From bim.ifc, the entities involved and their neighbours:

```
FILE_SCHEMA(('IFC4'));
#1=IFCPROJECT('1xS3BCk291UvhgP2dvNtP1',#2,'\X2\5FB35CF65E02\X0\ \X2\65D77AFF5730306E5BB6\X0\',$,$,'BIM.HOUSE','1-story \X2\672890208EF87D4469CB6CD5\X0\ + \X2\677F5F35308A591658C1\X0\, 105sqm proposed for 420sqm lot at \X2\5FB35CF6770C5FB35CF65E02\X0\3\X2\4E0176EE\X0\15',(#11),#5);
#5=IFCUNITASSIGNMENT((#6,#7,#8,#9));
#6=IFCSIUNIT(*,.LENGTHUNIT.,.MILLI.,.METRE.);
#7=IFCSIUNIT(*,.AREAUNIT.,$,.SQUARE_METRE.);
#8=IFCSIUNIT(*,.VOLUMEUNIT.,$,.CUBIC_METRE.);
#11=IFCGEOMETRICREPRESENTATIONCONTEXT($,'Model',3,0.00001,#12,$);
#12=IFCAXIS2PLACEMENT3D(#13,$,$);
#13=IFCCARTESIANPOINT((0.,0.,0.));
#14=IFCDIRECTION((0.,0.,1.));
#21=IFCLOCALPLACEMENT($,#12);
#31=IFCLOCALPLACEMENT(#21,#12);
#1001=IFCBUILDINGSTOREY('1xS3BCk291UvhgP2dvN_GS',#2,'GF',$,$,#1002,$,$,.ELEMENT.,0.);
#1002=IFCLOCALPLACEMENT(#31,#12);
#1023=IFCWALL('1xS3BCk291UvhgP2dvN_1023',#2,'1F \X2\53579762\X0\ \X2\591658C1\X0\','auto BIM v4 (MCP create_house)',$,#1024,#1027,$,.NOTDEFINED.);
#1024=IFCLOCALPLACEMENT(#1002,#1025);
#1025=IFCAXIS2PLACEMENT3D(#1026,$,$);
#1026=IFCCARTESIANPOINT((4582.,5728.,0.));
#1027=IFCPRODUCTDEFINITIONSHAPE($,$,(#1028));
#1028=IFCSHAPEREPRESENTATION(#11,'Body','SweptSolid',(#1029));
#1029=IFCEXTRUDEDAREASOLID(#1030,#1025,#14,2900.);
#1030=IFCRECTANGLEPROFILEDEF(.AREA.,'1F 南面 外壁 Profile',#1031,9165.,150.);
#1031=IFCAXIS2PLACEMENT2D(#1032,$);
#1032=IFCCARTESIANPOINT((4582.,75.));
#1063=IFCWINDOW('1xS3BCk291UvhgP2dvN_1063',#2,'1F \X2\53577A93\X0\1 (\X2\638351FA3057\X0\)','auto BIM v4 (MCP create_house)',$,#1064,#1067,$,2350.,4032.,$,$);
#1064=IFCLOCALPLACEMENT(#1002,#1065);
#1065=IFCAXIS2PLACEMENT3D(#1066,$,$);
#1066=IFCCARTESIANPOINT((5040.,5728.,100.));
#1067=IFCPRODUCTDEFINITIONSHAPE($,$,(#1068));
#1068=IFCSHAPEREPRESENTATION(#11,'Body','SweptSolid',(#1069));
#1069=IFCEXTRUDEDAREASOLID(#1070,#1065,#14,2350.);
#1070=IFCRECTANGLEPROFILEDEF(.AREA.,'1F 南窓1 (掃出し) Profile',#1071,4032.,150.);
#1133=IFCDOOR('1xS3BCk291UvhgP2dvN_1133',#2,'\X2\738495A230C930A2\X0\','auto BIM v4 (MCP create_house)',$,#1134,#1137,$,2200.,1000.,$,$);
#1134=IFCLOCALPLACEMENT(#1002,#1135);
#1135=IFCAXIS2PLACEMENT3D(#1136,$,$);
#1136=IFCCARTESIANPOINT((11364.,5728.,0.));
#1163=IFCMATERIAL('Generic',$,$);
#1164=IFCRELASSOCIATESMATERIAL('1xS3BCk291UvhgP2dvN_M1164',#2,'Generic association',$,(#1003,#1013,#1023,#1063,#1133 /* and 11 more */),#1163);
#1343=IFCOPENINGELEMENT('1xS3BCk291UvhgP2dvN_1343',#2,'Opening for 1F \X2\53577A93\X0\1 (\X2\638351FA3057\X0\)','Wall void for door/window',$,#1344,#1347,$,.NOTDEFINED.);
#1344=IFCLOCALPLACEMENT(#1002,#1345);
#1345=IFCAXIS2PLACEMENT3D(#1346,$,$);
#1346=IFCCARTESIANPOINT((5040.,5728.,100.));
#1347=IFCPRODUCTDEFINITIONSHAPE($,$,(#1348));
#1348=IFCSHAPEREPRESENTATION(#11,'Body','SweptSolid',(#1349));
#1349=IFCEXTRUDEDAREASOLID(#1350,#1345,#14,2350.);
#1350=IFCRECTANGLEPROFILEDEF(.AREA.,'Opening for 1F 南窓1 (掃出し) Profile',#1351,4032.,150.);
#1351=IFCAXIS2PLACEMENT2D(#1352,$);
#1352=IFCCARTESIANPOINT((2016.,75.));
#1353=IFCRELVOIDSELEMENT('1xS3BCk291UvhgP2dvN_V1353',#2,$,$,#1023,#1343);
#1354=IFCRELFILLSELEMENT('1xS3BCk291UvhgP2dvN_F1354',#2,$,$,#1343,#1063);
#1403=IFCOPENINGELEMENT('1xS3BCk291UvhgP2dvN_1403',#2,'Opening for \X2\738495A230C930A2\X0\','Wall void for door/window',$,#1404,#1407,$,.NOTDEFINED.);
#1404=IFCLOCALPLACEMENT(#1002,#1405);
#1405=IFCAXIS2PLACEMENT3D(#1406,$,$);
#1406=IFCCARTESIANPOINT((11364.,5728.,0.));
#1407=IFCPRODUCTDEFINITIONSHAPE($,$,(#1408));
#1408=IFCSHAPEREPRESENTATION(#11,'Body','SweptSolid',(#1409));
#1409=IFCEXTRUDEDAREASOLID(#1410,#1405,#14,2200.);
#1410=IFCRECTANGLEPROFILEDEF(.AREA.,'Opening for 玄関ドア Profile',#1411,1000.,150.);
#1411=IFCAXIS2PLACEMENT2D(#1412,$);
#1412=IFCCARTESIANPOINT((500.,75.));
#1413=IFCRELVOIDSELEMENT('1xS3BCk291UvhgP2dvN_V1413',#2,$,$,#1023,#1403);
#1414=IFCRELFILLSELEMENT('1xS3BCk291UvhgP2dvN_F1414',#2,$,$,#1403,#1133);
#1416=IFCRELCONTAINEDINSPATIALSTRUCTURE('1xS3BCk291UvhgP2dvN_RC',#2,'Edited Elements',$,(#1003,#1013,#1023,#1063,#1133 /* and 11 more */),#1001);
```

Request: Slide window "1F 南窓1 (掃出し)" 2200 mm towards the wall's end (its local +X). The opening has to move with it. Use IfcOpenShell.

```python
import ifcopenshell
import ifcopenshell.api.geometry
import ifcopenshell.util.placement
import ifcopenshell.util.unit

model = ifcopenshell.open("bim.ifc")
unit_scale = ifcopenshell.util.unit.calculate_unit_scale(model)

window = model.by_id(1063)
opening = window.FillsVoids[0].RelatingOpeningElement
wall = opening.VoidsElements[0].RelatingBuildingElement

wall_matrix = ifcopenshell.util.placement.get_local_placement(wall.ObjectPlacement)
shift = wall_matrix[:3, 0] * 2.2 / unit_scale
before = ifcopenshell.util.placement.get_local_placement(window.ObjectPlacement)[:3, 3].copy()

# The window is not placed relative to its opening, so move both.
for product in (opening, window):
    matrix = ifcopenshell.util.placement.get_local_placement(product.ObjectPlacement)
    matrix[:3, 3] += shift
    ifcopenshell.api.geometry.edit_object_placement(model, product=product, matrix=matrix, is_si=False)

after = ifcopenshell.util.placement.get_local_placement(window.ObjectPlacement)[:3, 3]
print("window moved by", (after - before).round(3) + 0.0)

model.write("bim_edited.ifc")
```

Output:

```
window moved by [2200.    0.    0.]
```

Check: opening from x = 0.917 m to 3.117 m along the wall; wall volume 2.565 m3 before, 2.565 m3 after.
